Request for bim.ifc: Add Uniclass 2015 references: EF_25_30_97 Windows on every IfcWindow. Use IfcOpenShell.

First a look at what the model holds.

```python
import ifcopenshell

model = ifcopenshell.open("bim.ifc")
print(model.schema)
print("classifications:", [c.Name for c in model.by_type("IfcClassification")])
for ifc_class in ("IfcDoor", "IfcRoof", "IfcStair", "IfcWall", "IfcWindow"):
    print(ifc_class, len(model.by_type(ifc_class)))
```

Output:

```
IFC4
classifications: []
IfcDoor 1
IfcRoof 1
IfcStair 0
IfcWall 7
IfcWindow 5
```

```python
import ifcopenshell
import ifcopenshell.api.classification

model = ifcopenshell.open("bim.ifc")

system = ifcopenshell.api.classification.add_classification(model, classification="Uniclass 2015")

codes = {
    "IfcWindow": ("EF_25_30_97", "Windows"),
}
for ifc_class, (code, name) in codes.items():
    products = model.by_type(ifc_class)
    ifcopenshell.api.classification.add_reference(
        model, products=products, classification=system, identification=code, name=name
    )
    print(code, len(products))

model.write("bim_updated.ifc")
```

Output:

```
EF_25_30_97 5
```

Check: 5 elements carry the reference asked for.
